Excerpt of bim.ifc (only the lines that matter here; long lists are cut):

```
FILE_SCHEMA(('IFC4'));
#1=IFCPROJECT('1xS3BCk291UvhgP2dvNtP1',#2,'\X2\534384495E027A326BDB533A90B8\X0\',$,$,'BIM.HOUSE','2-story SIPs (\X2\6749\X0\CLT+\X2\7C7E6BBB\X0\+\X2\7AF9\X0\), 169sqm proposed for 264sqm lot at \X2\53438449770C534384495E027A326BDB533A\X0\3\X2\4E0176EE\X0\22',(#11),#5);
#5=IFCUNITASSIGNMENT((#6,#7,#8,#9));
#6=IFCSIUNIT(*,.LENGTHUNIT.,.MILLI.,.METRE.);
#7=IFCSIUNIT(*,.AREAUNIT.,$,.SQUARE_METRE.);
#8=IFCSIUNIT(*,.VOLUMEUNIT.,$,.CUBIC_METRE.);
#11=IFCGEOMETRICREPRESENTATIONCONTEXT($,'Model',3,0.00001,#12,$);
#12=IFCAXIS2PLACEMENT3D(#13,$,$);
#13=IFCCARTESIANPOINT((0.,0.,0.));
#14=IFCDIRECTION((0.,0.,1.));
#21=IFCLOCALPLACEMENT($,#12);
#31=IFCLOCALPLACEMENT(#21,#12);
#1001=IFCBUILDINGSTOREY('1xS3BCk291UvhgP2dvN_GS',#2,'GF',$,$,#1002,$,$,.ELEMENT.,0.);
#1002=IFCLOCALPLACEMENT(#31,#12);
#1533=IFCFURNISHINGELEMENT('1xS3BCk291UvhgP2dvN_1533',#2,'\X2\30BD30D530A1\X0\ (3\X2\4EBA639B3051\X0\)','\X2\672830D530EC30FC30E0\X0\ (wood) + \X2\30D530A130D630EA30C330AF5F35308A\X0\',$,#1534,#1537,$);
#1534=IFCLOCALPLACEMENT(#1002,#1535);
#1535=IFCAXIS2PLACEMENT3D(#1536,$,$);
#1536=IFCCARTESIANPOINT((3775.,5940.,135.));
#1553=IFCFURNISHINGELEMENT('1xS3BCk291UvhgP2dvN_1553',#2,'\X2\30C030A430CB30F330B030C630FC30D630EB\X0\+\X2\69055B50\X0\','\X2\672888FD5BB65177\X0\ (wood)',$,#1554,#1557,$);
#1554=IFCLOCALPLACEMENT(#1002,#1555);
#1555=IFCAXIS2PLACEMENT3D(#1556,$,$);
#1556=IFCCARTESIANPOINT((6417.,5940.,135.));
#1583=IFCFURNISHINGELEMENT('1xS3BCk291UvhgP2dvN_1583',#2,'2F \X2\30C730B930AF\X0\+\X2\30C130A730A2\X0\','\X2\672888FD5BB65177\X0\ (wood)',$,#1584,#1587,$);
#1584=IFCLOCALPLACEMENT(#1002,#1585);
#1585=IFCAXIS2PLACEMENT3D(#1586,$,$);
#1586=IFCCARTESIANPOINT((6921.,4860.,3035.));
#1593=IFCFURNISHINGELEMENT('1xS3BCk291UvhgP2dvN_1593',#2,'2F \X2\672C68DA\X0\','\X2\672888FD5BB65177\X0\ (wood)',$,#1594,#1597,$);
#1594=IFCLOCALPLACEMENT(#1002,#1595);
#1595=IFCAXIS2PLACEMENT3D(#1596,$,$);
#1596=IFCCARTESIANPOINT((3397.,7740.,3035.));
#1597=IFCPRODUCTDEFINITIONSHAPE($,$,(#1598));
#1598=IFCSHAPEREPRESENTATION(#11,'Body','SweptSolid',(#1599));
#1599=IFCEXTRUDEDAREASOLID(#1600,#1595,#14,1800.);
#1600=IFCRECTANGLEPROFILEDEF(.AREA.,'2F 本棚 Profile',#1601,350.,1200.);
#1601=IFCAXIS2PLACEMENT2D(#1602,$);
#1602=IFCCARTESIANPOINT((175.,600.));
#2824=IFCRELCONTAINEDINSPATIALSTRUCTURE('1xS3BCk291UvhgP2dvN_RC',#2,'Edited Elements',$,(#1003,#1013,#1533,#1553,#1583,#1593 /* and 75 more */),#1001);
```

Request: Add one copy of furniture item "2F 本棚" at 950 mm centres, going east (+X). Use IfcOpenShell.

```python
import numpy as np
import ifcopenshell
import ifcopenshell.api.geometry
import ifcopenshell.api.root
import ifcopenshell.util.element
import ifcopenshell.util.placement
import ifcopenshell.util.unit

model = ifcopenshell.open("bim.ifc")
unit_scale = ifcopenshell.util.unit.calculate_unit_scale(model)


def reuse_history(source, copy):
    """copy_class also copies each property set's owner history, people and application; keep the originals."""
    for rel in copy.IsDefinedBy:
        if rel.is_a("IfcRelDefinesByProperties") and (history := rel.RelatingPropertyDefinition.OwnerHistory):
            rel.RelatingPropertyDefinition.OwnerHistory = source.OwnerHistory
            ifcopenshell.util.element.remove_deep2(model, history)


source = model.by_guid("1xS3BCk291UvhgP2dvN_1593")
base = ifcopenshell.util.placement.get_local_placement(source.ObjectPlacement)
step = np.array([1.0, 0.0, 0.0]) * 0.95 / unit_scale

for i in range(1, 2):
    copy = ifcopenshell.api.root.copy_class(model, product=source)
    copy.Representation = ifcopenshell.util.element.copy_deep(
        model, source.Representation, exclude=["IfcGeometricRepresentationContext", "IfcRepresentationMap"]
    )
    reuse_history(source, copy)
    matrix = base.copy()
    matrix[:3, 3] += i * step
    print("added at", matrix[:3, 3].round(3) + 0.0)
    ifcopenshell.api.geometry.edit_object_placement(model, product=copy, matrix=matrix, is_si=False)

model.write("bim_updated.ifc")
```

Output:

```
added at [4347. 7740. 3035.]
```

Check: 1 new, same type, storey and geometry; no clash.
